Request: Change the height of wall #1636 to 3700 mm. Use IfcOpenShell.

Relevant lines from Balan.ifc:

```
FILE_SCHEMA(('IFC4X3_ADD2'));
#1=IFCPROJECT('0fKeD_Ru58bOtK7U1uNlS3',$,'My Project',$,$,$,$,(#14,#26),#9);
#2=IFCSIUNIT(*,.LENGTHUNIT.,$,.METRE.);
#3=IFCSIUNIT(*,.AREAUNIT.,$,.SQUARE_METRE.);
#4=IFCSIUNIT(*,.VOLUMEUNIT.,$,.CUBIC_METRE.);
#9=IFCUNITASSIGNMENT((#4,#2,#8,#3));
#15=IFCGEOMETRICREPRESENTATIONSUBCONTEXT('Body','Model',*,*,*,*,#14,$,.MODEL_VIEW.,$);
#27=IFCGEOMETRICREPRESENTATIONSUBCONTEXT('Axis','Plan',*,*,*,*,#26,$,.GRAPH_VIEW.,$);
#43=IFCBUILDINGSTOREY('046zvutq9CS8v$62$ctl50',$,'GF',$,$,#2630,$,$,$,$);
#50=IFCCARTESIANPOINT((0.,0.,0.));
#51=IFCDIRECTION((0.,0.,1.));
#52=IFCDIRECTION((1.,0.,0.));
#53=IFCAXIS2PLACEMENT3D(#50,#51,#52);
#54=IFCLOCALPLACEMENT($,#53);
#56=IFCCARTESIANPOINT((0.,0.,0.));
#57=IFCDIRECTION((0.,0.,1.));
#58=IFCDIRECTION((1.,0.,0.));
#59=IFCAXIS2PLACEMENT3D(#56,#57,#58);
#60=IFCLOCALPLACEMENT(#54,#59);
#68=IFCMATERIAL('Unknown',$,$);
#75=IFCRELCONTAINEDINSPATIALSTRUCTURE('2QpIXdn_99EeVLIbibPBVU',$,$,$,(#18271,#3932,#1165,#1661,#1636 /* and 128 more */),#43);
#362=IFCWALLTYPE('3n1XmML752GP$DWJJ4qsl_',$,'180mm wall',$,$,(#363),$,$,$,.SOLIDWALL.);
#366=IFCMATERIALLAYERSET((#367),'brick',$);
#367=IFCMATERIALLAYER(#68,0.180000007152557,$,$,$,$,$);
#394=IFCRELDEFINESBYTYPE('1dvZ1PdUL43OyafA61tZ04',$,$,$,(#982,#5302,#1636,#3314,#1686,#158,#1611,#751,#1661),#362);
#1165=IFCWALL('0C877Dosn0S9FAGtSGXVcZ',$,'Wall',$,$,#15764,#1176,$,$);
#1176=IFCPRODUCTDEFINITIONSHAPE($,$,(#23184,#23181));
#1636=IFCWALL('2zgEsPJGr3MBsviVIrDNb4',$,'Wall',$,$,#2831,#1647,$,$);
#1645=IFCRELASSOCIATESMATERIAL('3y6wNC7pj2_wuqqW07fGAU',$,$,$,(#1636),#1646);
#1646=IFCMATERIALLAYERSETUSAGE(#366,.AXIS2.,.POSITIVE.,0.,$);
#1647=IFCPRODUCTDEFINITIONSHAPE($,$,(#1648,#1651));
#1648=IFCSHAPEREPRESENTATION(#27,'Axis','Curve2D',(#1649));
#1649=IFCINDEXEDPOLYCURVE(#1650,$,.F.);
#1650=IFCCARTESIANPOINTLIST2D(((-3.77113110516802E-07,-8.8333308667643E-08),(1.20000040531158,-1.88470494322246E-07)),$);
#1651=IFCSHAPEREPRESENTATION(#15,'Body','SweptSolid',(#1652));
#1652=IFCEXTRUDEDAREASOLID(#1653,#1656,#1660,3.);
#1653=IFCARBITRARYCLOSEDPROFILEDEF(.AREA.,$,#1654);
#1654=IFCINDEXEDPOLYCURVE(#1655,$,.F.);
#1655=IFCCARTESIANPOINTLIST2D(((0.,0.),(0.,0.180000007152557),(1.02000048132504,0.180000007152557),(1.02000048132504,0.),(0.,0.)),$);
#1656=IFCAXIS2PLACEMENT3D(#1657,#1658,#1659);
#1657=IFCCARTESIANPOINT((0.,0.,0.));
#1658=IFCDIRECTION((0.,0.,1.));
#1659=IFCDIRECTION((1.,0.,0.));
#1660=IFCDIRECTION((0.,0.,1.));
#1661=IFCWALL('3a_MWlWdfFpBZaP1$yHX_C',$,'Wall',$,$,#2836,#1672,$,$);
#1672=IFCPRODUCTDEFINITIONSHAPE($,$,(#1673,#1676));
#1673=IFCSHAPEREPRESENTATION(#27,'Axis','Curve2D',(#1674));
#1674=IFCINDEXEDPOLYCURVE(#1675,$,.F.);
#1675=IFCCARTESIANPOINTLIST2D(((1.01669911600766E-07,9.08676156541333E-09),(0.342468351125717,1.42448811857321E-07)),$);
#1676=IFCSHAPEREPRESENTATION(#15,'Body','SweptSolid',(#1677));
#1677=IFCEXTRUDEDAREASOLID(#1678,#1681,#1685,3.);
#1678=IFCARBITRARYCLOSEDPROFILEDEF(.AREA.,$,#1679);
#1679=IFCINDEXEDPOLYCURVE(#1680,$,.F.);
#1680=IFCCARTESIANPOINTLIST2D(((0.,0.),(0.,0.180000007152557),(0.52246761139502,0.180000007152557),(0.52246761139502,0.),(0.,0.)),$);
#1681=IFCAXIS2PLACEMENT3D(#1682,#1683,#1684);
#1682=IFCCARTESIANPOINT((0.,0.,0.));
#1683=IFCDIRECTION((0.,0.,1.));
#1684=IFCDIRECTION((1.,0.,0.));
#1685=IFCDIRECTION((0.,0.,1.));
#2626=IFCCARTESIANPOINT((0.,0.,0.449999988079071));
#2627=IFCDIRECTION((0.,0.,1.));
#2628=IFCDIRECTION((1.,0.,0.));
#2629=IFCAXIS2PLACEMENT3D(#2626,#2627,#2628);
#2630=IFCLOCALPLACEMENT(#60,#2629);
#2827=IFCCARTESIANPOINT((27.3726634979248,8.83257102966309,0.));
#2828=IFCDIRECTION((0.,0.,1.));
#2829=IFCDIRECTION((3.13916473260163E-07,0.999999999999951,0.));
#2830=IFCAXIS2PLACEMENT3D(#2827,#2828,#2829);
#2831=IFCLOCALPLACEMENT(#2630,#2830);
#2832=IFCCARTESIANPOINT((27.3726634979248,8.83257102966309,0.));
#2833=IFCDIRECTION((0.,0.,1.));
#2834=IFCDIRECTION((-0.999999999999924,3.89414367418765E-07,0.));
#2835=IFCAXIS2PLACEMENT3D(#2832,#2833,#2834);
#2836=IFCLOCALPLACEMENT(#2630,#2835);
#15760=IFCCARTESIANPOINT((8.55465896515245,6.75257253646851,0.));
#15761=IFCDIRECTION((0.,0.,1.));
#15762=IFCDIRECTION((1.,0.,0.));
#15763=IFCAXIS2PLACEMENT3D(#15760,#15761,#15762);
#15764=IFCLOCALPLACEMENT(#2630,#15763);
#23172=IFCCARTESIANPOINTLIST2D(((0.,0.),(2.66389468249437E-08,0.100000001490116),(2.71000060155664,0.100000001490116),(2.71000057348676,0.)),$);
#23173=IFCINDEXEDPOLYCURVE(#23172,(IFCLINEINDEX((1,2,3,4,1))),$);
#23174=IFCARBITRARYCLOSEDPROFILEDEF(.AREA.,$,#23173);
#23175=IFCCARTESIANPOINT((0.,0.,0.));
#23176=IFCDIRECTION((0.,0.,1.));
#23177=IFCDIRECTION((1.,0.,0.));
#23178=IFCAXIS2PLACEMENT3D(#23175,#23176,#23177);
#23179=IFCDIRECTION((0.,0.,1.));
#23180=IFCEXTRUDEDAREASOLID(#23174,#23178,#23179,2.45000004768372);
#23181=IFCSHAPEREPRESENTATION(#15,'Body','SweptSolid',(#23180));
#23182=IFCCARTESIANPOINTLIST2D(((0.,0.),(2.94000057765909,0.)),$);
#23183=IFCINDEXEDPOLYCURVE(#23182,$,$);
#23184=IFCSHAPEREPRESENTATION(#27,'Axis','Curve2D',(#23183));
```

```python
import ifcopenshell
import ifcopenshell.geom
import ifcopenshell.util.representation
import ifcopenshell.util.shape
import ifcopenshell.util.unit

model = ifcopenshell.open("Balan.ifc")
unit_scale = ifcopenshell.util.unit.calculate_unit_scale(model)
settings = ifcopenshell.geom.settings()


def volume(element):
    """Net volume in cubic metres, openings subtracted."""
    shape = ifcopenshell.geom.create_shape(settings, element)
    return ifcopenshell.util.shape.get_volume(shape.geometry)


wall = model.by_guid("2zgEsPJGr3MBsviVIrDNb4")
before = volume(wall)

body = ifcopenshell.util.representation.get_representation(wall, "Model", "Body")
solid = body.Items[0]
old_height = solid.Depth
solid.Depth = 3.7 / unit_scale
after = volume(wall)

print(f"height {old_height:g} -> {solid.Depth:g}, volume {before:.3f} -> {after:.3f} m3")

model.write("Balan_v2.ifc")
```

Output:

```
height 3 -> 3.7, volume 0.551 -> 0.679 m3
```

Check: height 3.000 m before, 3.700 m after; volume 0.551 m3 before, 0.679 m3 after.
